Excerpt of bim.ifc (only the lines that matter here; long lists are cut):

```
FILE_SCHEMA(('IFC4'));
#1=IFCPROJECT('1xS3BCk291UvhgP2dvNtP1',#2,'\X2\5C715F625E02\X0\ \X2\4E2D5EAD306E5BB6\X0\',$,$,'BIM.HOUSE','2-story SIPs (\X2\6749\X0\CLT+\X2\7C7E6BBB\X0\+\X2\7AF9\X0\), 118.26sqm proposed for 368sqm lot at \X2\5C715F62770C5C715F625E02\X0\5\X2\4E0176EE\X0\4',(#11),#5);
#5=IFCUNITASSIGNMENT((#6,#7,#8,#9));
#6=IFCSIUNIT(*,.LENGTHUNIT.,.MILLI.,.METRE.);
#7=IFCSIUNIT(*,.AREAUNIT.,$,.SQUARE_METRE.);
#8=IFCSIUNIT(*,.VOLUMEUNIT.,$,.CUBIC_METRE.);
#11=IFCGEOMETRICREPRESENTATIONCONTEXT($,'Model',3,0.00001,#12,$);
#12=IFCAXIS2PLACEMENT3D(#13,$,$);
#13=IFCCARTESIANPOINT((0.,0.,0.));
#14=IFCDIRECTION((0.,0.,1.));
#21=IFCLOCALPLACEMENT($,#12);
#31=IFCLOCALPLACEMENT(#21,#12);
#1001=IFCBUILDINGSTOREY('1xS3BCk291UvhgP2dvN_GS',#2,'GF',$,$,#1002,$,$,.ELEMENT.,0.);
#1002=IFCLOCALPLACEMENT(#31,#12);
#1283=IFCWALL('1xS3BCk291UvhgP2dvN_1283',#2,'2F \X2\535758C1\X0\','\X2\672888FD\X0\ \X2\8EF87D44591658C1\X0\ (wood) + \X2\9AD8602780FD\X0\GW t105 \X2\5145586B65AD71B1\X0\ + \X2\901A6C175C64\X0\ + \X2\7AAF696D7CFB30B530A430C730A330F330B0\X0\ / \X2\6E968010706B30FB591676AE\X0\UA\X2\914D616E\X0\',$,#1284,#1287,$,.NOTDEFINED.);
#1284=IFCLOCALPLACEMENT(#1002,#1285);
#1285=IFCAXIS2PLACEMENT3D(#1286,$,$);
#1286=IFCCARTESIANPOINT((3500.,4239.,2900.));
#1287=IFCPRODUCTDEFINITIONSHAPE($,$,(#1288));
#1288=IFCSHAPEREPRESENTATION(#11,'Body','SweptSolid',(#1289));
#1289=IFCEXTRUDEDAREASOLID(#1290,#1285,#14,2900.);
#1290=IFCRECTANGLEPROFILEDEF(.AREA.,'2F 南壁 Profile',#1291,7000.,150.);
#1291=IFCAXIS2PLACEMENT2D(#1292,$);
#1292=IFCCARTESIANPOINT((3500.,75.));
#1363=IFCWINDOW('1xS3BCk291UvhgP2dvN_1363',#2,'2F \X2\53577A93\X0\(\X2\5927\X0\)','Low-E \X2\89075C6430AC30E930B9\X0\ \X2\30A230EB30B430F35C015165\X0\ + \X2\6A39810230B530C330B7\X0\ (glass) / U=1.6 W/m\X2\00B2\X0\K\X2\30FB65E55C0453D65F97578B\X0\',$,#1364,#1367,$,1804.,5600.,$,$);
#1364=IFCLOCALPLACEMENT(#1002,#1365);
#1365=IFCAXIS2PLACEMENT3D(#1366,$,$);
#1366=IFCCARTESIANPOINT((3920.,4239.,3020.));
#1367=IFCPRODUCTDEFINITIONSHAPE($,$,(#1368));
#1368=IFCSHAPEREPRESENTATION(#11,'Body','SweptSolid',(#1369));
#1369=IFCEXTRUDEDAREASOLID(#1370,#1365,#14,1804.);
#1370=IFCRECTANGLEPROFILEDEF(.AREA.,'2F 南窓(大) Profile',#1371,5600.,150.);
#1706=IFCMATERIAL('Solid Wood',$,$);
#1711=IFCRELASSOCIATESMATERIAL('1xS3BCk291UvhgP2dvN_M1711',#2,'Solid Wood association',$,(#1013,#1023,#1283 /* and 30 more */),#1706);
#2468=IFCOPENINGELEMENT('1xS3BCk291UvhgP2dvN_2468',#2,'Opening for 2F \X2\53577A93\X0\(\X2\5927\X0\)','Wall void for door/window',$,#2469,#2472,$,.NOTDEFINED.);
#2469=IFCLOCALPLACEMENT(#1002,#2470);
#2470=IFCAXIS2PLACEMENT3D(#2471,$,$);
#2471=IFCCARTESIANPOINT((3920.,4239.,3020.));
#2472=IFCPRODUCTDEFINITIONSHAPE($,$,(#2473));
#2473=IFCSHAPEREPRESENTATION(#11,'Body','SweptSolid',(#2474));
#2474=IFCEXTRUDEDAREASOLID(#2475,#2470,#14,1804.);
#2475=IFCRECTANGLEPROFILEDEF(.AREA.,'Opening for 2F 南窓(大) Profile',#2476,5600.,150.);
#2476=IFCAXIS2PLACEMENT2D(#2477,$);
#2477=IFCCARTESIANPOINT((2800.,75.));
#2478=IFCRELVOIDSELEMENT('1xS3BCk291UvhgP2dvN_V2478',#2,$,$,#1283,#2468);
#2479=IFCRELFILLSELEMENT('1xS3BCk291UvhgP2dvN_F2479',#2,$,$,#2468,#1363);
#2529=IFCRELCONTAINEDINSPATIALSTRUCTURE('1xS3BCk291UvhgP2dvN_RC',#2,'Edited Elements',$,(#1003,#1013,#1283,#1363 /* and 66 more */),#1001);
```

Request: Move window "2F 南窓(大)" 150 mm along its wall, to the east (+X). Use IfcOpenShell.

```python
import ifcopenshell
import ifcopenshell.api.geometry
import ifcopenshell.util.placement

model = ifcopenshell.open("bim.ifc")

window = model.by_guid("1xS3BCk291UvhgP2dvN_1363")
opening = window.FillsVoids[0].RelatingOpeningElement
wall = opening.VoidsElements[0].RelatingBuildingElement

wall_matrix = ifcopenshell.util.placement.get_local_placement(wall.ObjectPlacement)
shift = wall_matrix[:3, 0] * 150.0
before = ifcopenshell.util.placement.get_local_placement(window.ObjectPlacement)[:3, 3].copy()

# The window is not placed relative to its opening, so move both.
for product in (opening, window):
    matrix = ifcopenshell.util.placement.get_local_placement(product.ObjectPlacement)
    matrix[:3, 3] += shift
    ifcopenshell.api.geometry.edit_object_placement(model, product=product, matrix=matrix, is_si=False)

after = ifcopenshell.util.placement.get_local_placement(window.ObjectPlacement)[:3, 3]
print("window moved by", (after - before).round(3) + 0.0)

model.write("bim_updated.ifc")
```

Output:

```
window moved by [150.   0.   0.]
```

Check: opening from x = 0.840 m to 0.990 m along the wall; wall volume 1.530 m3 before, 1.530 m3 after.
